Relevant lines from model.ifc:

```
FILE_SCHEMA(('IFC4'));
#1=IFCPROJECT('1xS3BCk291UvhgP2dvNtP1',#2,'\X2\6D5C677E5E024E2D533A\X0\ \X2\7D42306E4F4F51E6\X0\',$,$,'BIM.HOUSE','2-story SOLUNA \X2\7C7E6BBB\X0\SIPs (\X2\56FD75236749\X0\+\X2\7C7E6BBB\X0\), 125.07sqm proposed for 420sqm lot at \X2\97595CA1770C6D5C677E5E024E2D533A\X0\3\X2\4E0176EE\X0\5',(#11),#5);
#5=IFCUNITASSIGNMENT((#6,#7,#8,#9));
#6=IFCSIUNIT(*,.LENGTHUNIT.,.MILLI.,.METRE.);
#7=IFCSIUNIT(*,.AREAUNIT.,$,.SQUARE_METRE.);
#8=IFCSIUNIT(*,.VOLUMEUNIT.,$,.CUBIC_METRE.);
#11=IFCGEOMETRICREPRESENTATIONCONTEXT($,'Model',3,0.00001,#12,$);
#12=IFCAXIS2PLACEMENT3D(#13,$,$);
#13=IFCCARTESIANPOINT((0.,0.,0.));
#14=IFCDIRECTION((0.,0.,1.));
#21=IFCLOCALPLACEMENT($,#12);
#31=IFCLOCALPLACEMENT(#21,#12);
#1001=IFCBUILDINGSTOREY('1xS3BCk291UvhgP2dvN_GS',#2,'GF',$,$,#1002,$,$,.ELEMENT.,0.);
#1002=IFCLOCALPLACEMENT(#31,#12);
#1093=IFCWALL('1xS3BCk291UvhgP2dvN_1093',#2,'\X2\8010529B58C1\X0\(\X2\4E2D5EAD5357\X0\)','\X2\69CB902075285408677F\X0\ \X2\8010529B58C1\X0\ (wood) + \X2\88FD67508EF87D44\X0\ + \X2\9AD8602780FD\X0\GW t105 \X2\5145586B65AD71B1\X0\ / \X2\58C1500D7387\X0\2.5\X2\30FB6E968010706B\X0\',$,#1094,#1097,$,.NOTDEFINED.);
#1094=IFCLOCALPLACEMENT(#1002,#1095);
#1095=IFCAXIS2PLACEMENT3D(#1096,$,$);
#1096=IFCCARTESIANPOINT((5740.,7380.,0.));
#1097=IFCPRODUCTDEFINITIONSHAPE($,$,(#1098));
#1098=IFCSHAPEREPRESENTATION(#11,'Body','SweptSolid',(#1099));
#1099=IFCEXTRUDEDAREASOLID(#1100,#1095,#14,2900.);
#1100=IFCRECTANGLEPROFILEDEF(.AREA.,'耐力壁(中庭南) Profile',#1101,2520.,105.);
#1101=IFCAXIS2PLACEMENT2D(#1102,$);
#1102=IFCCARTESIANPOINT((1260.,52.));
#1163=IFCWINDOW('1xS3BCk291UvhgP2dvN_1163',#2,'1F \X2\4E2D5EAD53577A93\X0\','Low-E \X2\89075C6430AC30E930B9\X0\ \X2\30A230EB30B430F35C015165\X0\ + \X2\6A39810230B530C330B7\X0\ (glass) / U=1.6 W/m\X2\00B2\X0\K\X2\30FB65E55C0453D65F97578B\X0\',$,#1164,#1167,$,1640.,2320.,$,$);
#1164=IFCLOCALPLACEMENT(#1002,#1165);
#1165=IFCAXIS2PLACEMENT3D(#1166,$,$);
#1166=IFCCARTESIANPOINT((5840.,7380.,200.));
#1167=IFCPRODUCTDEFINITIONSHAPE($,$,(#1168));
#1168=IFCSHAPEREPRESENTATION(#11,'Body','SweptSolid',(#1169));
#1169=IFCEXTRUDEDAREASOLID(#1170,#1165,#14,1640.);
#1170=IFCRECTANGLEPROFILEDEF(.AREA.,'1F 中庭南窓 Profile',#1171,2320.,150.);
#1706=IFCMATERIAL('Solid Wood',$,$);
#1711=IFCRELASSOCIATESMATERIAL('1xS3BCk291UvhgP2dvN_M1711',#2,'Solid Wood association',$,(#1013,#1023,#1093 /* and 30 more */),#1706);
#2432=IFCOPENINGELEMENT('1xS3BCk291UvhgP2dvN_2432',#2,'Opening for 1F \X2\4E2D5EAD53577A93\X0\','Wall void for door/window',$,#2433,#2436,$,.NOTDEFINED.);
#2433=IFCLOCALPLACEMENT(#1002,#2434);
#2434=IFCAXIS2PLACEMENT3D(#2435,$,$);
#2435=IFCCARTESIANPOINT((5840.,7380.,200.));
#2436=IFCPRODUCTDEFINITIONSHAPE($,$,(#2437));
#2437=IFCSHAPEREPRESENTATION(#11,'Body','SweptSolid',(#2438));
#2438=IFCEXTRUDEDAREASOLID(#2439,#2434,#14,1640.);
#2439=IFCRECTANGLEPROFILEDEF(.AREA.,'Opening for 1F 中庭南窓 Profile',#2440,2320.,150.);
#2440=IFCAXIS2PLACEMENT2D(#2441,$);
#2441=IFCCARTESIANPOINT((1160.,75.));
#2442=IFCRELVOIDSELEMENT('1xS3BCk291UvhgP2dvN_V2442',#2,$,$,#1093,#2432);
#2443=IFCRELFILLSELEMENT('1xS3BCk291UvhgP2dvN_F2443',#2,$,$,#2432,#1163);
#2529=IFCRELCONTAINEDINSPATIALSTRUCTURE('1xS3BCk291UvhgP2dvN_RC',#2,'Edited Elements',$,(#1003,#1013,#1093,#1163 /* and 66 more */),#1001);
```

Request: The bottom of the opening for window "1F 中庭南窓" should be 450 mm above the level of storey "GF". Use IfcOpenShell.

```python
import numpy as np
import ifcopenshell
import ifcopenshell.api.geometry
import ifcopenshell.geom
import ifcopenshell.util.element
import ifcopenshell.util.placement
import ifcopenshell.util.shape
import ifcopenshell.util.unit

model = ifcopenshell.open("model.ifc")
unit_scale = ifcopenshell.util.unit.calculate_unit_scale(model)

window = model.by_guid("1xS3BCk291UvhgP2dvN_1163")
opening = window.FillsVoids[0].RelatingOpeningElement
storey = ifcopenshell.util.element.get_container(window, ifc_class="IfcBuildingStorey")
level = ifcopenshell.util.placement.get_local_placement(storey.ObjectPlacement)[2, 3]

# The opening's origin need not be at the sill, so measure its lowest point.
shape = ifcopenshell.geom.create_shape(ifcopenshell.geom.settings(), opening)
bottom = ifcopenshell.util.shape.get_shape_bottom_elevation(shape, shape.geometry) / unit_scale
dz = level + 450.0 - bottom

shift = np.array([0.0, 0.0, dz])
# The window is not placed relative to its opening, so move both.
for product in (opening, window):
    matrix = ifcopenshell.util.placement.get_local_placement(product.ObjectPlacement)
    matrix[:3, 3] += shift
    ifcopenshell.api.geometry.edit_object_placement(model, product=product, matrix=matrix, is_si=False)

print(f"moved by {dz * unit_scale:+.3f} m")

model.write("model_edited.ifc")
```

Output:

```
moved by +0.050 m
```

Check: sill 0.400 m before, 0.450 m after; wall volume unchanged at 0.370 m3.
